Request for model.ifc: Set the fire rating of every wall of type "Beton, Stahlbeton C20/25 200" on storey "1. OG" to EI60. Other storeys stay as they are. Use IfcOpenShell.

First a look at what the model holds.

```python
import ifcopenshell
import ifcopenshell.util.element

model = ifcopenshell.open("model.ifc")
print(model.schema)
storey = next(s for s in model.by_type("IfcBuildingStorey") if s.Name == "1. OG")
walls = [e for e in ifcopenshell.util.element.get_decomposition(storey) if e.is_a("IfcWall")]
seen = {}
for e in walls:
    element_type = ifcopenshell.util.element.get_type(e)
    key = (element_type.Name if element_type != e and element_type else None, ifcopenshell.util.element.get_pset(e, "Pset_WallCommon", "FireRating"))
    seen[key] = seen.get(key, 0) + 1
for (name, value), count in sorted(seen.items(), key=str):
    print(count, "x", name, "|", value)
```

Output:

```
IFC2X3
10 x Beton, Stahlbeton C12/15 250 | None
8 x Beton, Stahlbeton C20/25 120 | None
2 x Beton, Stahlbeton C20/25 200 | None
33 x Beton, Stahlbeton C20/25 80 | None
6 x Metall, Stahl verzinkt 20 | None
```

```python
import ifcopenshell
import ifcopenshell.api.pset
import ifcopenshell.util.element

model = ifcopenshell.open("model.ifc")

storey = next(s for s in model.by_type("IfcBuildingStorey") if s.Name == "1. OG")
walls = [e for e in ifcopenshell.util.element.get_decomposition(storey) if e.is_a("IfcWall")]

count = 0
for e in walls:
    element_type = ifcopenshell.util.element.get_type(e)
    if element_type in (None, e) or element_type.Name != "Beton, Stahlbeton C20/25 200":
        continue
    # add_pset returns the element's existing set when there is one.
    pset = ifcopenshell.api.pset.add_pset(model, product=e, name="Pset_WallCommon")
    ifcopenshell.api.pset.edit_pset(model, pset=pset, properties={"FireRating": "EI60"})
    count += 1

print(count, "walls updated")

model.write("model-out.ifc")
```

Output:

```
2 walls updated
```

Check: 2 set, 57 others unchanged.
